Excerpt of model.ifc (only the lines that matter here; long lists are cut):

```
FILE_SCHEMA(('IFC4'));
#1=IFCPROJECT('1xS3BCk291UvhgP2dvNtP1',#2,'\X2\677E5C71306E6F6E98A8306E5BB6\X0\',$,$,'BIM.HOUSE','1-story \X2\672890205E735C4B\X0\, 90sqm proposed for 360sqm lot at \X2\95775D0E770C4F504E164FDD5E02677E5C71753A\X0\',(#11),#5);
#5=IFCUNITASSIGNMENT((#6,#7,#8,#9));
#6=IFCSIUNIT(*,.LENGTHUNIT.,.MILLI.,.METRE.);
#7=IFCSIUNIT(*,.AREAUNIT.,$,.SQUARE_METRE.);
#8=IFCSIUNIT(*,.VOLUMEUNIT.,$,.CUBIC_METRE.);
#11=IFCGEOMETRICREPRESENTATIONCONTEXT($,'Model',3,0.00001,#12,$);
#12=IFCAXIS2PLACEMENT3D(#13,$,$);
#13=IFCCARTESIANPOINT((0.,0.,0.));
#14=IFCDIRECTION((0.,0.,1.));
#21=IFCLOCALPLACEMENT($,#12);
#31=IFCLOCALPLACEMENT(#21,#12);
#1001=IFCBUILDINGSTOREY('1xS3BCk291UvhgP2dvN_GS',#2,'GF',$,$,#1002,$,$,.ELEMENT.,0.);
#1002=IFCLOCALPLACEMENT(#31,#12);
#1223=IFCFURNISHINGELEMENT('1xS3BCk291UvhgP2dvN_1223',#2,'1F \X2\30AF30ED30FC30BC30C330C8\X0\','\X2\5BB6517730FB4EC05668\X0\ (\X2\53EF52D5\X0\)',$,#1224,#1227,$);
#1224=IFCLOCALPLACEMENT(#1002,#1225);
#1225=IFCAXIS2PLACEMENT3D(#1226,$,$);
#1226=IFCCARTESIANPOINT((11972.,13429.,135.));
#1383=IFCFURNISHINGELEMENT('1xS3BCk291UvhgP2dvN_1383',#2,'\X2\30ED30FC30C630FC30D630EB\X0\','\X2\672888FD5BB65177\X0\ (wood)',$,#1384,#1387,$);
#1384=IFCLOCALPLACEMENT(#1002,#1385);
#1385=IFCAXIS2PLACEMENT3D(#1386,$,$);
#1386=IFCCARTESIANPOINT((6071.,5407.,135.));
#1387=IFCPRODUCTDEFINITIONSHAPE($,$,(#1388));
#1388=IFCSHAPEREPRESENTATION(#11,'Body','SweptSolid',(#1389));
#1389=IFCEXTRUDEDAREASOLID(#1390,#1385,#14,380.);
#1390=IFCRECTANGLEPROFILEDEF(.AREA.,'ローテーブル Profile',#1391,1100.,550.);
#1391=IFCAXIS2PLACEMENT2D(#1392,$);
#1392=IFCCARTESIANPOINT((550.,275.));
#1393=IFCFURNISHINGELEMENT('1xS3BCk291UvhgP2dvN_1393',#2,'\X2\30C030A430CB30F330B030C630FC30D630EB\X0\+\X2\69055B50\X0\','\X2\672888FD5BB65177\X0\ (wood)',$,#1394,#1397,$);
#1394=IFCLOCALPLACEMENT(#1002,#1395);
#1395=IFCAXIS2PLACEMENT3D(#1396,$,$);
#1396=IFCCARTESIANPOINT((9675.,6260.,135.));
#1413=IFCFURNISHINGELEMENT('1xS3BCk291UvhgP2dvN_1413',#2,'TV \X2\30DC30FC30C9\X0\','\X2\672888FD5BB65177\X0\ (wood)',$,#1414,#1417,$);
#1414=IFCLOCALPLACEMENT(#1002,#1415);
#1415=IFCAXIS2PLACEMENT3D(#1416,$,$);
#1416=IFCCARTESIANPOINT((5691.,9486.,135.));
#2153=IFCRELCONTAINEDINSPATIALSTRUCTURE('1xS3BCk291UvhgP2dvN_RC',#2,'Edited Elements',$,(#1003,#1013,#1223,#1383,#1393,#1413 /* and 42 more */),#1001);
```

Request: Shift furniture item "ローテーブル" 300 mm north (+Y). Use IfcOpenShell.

```python
import ifcopenshell
import ifcopenshell.api.geometry
import ifcopenshell.util.placement

model = ifcopenshell.open("model.ifc")

item = model.by_id(1383)
matrix = ifcopenshell.util.placement.get_local_placement(item.ObjectPlacement)
matrix[1, 3] += 300.0
ifcopenshell.api.geometry.edit_object_placement(model, product=item, matrix=matrix, is_si=False)

print(ifcopenshell.util.placement.get_local_placement(item.ObjectPlacement).round(3) + 0.0)

model.write("model_edited.ifc")
```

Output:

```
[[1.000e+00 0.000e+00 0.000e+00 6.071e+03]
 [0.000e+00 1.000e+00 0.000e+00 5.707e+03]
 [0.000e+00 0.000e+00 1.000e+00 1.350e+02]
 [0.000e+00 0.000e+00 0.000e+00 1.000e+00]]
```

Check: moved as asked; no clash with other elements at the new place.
